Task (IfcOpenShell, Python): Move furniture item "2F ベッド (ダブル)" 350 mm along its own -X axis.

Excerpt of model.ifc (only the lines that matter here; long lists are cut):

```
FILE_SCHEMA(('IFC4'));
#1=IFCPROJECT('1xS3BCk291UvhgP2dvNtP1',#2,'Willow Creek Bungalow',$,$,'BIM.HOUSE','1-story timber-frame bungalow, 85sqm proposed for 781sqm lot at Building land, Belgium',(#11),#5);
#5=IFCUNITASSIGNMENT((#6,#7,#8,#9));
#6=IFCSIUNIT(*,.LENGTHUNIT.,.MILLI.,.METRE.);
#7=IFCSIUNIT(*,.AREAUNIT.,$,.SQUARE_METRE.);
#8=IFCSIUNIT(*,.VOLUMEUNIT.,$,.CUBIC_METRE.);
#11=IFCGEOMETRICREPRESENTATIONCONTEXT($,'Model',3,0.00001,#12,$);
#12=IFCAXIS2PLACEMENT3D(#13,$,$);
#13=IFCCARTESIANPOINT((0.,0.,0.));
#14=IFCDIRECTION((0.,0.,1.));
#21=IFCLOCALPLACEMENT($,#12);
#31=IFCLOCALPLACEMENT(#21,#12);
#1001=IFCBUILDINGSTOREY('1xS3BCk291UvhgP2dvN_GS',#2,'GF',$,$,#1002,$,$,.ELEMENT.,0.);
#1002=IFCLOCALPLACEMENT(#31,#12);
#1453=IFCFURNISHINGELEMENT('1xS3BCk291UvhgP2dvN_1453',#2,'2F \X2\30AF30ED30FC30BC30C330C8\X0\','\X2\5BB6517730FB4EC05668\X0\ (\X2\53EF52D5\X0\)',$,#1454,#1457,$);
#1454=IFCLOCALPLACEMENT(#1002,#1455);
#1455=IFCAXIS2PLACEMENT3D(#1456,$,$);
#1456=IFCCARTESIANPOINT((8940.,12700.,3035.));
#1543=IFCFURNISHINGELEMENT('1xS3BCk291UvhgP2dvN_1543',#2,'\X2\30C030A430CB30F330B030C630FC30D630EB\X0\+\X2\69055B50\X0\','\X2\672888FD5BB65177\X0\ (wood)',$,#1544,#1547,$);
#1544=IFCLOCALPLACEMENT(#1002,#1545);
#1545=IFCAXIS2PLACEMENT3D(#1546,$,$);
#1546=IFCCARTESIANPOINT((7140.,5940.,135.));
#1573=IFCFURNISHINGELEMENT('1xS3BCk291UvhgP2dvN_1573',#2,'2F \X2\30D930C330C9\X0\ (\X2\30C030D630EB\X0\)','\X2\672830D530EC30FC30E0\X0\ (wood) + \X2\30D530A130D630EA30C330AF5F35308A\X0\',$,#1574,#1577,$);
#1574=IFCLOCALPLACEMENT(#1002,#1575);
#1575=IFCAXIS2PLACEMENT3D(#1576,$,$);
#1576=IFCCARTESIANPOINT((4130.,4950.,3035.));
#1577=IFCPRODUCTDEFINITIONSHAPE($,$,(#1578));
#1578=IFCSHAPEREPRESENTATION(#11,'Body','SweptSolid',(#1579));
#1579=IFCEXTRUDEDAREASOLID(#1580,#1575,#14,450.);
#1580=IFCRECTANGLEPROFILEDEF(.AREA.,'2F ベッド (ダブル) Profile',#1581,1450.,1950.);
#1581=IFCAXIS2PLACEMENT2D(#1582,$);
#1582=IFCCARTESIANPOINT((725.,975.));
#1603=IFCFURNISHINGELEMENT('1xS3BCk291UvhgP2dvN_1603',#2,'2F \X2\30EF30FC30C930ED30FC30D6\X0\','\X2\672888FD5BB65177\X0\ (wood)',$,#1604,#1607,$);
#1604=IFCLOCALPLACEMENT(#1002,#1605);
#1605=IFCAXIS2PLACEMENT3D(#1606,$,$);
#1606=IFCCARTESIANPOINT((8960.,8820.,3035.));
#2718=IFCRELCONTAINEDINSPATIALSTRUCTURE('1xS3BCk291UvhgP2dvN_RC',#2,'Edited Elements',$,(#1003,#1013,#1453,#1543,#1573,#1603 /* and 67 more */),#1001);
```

```python
import ifcopenshell
import ifcopenshell.api.geometry
import ifcopenshell.util.placement

model = ifcopenshell.open("model.ifc")

item = model.by_guid("1xS3BCk291UvhgP2dvN_1573")
matrix = ifcopenshell.util.placement.get_local_placement(item.ObjectPlacement)
matrix[:3, 3] -= matrix[:3, 0] * 350.0
ifcopenshell.api.geometry.edit_object_placement(model, product=item, matrix=matrix, is_si=False)

print(ifcopenshell.util.placement.get_local_placement(item.ObjectPlacement).round(3) + 0.0)

model.write("model_v2.ifc")
```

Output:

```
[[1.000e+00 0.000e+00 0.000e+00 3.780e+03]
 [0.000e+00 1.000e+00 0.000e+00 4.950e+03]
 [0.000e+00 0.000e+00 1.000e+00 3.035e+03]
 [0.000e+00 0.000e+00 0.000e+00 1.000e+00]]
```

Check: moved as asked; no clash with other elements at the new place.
